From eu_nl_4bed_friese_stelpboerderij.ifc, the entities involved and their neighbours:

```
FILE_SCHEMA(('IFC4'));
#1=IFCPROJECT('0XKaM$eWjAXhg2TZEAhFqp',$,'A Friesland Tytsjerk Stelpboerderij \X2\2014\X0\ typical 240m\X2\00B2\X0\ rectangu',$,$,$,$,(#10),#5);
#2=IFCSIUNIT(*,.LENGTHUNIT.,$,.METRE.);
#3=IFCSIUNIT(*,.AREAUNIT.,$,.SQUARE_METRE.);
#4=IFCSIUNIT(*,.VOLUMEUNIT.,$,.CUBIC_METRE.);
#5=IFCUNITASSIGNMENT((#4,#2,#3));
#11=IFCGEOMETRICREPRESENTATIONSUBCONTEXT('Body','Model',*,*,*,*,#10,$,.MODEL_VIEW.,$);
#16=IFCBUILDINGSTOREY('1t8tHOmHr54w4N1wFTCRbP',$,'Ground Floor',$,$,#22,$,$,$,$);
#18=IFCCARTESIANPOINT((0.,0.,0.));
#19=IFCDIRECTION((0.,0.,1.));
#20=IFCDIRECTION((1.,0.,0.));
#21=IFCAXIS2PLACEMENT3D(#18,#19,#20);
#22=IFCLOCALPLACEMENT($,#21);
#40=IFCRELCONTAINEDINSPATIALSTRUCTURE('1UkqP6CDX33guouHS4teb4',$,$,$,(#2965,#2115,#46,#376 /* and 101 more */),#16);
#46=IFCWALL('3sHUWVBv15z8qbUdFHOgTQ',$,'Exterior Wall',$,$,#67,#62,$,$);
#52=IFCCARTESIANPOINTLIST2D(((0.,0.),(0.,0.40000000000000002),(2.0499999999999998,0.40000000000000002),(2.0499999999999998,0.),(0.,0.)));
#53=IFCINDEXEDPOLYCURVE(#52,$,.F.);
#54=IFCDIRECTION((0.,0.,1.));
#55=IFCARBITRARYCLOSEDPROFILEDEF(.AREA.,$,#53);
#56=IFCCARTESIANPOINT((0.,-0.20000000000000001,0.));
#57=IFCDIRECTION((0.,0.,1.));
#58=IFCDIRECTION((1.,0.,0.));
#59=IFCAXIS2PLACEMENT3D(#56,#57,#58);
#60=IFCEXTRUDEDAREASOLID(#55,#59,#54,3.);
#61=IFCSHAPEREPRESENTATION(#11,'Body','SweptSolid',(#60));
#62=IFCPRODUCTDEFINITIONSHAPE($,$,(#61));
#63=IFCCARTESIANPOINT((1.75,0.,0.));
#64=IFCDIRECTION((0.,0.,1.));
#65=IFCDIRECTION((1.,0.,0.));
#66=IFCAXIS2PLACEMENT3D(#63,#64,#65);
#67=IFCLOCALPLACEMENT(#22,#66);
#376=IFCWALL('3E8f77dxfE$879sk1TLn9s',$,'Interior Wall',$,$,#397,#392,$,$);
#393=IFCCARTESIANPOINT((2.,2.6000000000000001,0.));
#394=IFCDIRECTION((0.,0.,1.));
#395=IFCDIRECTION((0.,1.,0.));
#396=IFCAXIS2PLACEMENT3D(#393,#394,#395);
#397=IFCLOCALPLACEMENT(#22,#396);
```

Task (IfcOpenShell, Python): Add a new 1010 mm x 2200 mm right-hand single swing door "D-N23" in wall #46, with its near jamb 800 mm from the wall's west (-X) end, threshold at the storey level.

```python
import numpy as np
import ifcopenshell
import ifcopenshell.api.feature
import ifcopenshell.api.geometry
import ifcopenshell.api.root
import ifcopenshell.api.spatial
import ifcopenshell.geom
import ifcopenshell.util.element
import ifcopenshell.util.placement
import ifcopenshell.util.representation
import ifcopenshell.util.shape
import ifcopenshell.util.unit

model = ifcopenshell.open("eu_nl_4bed_friese_stelpboerderij.ifc")
unit_scale = ifcopenshell.util.unit.calculate_unit_scale(model)
settings = ifcopenshell.geom.settings()


def volume(element):
    """Net volume in cubic metres, openings subtracted."""
    shape = ifcopenshell.geom.create_shape(settings, element)
    return ifcopenshell.util.shape.get_volume(shape.geometry)


wall = model.by_guid("3sHUWVBv15z8qbUdFHOgTQ")
storey = ifcopenshell.util.element.get_container(wall, ifc_class="IfcBuildingStorey")
context = ifcopenshell.util.representation.get_context(model, "Model", "Body", "MODEL_VIEW")
before = volume(wall)

width, height, from_end, sill = 1.01, 2.2, 0.8, 0.0  # metres

# The wall runs along its own X axis, and the end named is its -X end.
wall_shape = ifcopenshell.geom.create_shape(settings, wall)
x, y, z = ifcopenshell.util.shape.get_vertices(wall_shape.geometry).T
start = x.min() + from_end
face, thickness = float(y.min()), float(y.max() - y.min())
wall_matrix = ifcopenshell.util.placement.get_local_placement(wall.ObjectPlacement)
level = ifcopenshell.util.placement.get_local_placement(storey.ObjectPlacement)[2, 3]


def in_wall(x, y):
    """Placement at x, y metres in the wall's axes, at sill height."""
    matrix = wall_matrix.copy()
    matrix[:, 3] = wall_matrix @ np.array([x / unit_scale, y / unit_scale, 0.0, 1.0])
    matrix[2, 3] = level + sill / unit_scale
    return matrix


# Opening: a box that overshoots both wall faces by 50 mm.
opening = ifcopenshell.api.root.create_entity(model, ifc_class="IfcOpeningElement", predefined_type="OPENING")
box = ifcopenshell.api.geometry.add_wall_representation(
    model, context=context, length=width, height=height, thickness=thickness + 0.1
)
ifcopenshell.api.geometry.assign_representation(model, product=opening, representation=box)
ifcopenshell.api.geometry.edit_object_placement(model, product=opening, matrix=in_wall(start, face - 0.05), is_si=False)
ifcopenshell.api.feature.add_feature(model, feature=opening, element=wall)

door = ifcopenshell.api.root.create_entity(model, ifc_class="IfcDoor", name="D-N23", predefined_type="DOOR")
door.OverallWidth, door.OverallHeight = width / unit_scale, height / unit_scale
door.OperationType = "SINGLE_SWING_RIGHT"
body = ifcopenshell.api.geometry.add_door_representation(
    model,
    context=context,
    overall_width=door.OverallWidth,
    overall_height=door.OverallHeight,
    operation_type="SINGLE_SWING_RIGHT",
    lining_properties={"LiningDepth": thickness / unit_scale, "ThresholdDepth": thickness / unit_scale},
)
ifcopenshell.api.geometry.assign_representation(model, product=door, representation=body)
ifcopenshell.api.spatial.assign_container(model, products=[door], relating_structure=storey)
ifcopenshell.api.feature.add_filling(model, opening=opening, element=door)

# The lining spans the wall, so the door starts at the wall face.
ifcopenshell.api.geometry.edit_object_placement(model, product=door, matrix=in_wall(start, face), is_si=False)

after = volume(wall)

print(f"wall volume {before:.3f} -> {after:.3f} m3")

model.write("eu_nl_4bed_friese_stelpboerderij_edited.ifc")
```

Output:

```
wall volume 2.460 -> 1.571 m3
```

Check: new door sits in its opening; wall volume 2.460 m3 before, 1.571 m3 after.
